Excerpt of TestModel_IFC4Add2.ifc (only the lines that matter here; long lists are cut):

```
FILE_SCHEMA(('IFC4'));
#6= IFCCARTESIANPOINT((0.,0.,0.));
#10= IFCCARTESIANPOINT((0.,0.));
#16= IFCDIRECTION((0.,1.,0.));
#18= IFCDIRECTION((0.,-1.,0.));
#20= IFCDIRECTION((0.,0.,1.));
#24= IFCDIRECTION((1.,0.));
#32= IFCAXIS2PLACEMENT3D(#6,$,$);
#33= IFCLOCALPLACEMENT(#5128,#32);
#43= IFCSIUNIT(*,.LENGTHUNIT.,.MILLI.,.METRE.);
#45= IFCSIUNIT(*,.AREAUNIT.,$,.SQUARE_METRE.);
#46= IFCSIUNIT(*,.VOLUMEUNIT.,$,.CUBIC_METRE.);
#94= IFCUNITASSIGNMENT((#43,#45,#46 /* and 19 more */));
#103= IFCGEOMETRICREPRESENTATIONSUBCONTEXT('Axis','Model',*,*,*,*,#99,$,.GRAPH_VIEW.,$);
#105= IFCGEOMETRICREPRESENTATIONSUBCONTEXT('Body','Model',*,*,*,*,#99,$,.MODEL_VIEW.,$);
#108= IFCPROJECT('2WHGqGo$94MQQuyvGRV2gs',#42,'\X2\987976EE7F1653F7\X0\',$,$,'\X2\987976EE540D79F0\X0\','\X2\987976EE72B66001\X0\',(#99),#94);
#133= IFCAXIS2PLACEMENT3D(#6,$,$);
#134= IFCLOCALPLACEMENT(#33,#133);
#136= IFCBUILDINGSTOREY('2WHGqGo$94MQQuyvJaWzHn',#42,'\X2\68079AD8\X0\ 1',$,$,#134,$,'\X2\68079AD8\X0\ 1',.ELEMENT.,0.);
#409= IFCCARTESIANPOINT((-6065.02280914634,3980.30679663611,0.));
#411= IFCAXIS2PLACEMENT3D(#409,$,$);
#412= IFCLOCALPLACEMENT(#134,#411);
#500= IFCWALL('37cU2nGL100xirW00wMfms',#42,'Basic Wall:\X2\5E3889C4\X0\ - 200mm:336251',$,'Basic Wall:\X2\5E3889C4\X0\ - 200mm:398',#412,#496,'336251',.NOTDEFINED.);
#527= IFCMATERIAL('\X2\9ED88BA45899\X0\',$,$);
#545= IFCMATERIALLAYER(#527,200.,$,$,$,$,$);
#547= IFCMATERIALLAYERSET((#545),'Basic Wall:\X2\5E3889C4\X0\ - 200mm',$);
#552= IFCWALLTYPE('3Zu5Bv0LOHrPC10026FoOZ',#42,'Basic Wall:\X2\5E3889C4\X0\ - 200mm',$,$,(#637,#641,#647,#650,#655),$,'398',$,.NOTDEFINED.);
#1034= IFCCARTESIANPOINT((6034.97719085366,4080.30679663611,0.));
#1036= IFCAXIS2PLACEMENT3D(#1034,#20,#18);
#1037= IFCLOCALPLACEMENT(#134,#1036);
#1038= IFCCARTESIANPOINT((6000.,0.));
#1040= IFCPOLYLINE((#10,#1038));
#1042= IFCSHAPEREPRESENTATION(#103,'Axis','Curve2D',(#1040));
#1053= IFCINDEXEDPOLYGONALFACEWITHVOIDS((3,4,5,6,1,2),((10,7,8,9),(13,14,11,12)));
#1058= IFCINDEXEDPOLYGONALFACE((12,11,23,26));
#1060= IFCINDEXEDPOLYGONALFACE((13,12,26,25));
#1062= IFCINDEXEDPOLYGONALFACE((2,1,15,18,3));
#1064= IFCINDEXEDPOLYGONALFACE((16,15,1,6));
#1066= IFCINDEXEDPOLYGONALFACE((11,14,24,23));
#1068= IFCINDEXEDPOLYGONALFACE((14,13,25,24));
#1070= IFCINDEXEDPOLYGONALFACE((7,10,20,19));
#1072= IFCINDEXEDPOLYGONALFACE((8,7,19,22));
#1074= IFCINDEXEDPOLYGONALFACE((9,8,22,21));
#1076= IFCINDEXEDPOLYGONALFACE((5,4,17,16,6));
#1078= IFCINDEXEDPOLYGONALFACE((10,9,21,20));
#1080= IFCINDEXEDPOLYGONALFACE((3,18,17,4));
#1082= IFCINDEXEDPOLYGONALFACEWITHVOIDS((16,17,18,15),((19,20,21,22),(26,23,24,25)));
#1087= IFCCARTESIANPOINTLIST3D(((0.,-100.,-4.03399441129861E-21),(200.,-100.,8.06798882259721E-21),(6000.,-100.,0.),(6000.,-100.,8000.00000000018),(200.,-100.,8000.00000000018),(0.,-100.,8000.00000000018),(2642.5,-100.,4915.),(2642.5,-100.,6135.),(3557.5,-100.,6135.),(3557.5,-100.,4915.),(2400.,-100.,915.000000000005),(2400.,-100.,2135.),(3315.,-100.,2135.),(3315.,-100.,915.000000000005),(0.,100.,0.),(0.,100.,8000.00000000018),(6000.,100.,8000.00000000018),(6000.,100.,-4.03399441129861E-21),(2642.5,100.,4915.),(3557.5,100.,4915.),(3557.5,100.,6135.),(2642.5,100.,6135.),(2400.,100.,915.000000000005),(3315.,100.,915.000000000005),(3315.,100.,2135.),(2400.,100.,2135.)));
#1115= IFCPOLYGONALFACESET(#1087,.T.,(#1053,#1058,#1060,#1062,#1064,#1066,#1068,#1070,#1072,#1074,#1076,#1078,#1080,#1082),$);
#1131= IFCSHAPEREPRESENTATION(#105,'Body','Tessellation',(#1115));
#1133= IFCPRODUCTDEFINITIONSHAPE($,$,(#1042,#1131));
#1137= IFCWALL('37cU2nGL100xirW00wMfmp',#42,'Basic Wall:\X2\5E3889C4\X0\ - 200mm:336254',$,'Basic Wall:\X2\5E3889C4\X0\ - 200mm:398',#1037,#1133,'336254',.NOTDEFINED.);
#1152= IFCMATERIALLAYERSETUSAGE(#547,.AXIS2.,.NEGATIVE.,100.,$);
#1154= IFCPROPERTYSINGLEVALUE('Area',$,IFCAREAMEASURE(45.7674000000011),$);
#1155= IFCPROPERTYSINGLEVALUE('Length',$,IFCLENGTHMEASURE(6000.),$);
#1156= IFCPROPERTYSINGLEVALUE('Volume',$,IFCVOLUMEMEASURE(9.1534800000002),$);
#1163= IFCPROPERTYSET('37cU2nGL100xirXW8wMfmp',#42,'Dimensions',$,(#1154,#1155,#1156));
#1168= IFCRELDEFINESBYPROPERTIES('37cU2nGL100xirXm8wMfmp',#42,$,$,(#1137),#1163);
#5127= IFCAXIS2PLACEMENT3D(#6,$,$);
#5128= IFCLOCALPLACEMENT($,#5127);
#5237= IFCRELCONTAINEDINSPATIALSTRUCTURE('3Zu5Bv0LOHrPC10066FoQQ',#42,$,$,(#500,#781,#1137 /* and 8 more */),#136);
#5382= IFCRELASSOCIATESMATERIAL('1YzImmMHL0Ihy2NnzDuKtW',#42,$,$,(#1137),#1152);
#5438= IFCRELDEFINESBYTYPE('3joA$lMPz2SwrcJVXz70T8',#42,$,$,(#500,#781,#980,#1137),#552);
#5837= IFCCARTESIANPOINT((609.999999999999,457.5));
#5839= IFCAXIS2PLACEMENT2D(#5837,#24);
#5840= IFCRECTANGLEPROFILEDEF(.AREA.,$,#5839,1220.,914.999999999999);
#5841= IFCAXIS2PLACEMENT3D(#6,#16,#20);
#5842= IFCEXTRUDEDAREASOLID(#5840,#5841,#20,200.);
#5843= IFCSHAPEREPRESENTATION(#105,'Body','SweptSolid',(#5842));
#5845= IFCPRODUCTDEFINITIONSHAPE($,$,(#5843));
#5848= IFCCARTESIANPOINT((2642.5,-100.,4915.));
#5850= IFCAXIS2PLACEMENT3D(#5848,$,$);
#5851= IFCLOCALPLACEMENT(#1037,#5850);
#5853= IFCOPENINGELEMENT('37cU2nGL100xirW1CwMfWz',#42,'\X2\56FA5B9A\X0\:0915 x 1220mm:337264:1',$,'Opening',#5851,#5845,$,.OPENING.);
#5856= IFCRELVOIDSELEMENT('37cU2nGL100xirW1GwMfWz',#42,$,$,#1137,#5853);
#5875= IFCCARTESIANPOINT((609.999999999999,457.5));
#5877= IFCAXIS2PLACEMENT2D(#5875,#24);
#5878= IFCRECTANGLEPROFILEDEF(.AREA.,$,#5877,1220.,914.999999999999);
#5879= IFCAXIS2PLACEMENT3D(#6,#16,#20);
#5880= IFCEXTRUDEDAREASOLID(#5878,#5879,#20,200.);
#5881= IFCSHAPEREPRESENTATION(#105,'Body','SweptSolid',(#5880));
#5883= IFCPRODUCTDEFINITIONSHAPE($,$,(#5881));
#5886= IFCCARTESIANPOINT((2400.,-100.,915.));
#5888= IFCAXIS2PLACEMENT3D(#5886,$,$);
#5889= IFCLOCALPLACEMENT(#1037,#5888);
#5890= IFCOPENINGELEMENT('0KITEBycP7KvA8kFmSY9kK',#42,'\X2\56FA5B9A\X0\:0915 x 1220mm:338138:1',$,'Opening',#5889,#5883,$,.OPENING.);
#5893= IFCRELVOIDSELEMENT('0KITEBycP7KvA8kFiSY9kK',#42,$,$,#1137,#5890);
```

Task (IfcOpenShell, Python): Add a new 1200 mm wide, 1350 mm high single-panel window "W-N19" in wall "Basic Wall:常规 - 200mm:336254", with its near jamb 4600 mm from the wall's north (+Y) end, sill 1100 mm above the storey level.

```python
import numpy as np
import ifcopenshell
import ifcopenshell.api.feature
import ifcopenshell.api.geometry
import ifcopenshell.api.pset
import ifcopenshell.api.root
import ifcopenshell.api.spatial
import ifcopenshell.geom
import ifcopenshell.util.element
import ifcopenshell.util.placement
import ifcopenshell.util.representation
import ifcopenshell.util.shape
import ifcopenshell.util.unit

model = ifcopenshell.open("TestModel_IFC4Add2.ifc")
unit_scale = ifcopenshell.util.unit.calculate_unit_scale(model)
area_scale = ifcopenshell.util.unit.calculate_unit_scale(model, "AREAUNIT")
volume_scale = ifcopenshell.util.unit.calculate_unit_scale(model, "VOLUMEUNIT")
settings = ifcopenshell.geom.settings()


def volume(element):
    """Net volume in cubic metres, openings subtracted."""
    shape = ifcopenshell.geom.create_shape(settings, element)
    return ifcopenshell.util.shape.get_volume(shape.geometry)


wall = model.by_guid("37cU2nGL100xirW00wMfmp")
storey = ifcopenshell.util.element.get_container(wall, ifc_class="IfcBuildingStorey")
context = ifcopenshell.util.representation.get_context(model, "Model", "Body", "MODEL_VIEW")
before = volume(wall)

width, height, from_end, sill = 1.2, 1.35, 4.6, 1.1  # metres

# The wall runs along its own X axis, and the end named is its -X end.
wall_shape = ifcopenshell.geom.create_shape(settings, wall)
x, y, z = ifcopenshell.util.shape.get_vertices(wall_shape.geometry).T
start = x.min() + from_end
face, thickness = float(y.min()), float(y.max() - y.min())
wall_matrix = ifcopenshell.util.placement.get_local_placement(wall.ObjectPlacement)
level = ifcopenshell.util.placement.get_local_placement(storey.ObjectPlacement)[2, 3]


def in_wall(x, y):
    """Placement at x, y metres in the wall's axes, at sill height."""
    matrix = wall_matrix.copy()
    matrix[:, 3] = wall_matrix @ np.array([x / unit_scale, y / unit_scale, 0.0, 1.0])
    matrix[2, 3] = level + sill / unit_scale
    return matrix


# Opening: a box that overshoots both wall faces by 50 mm.
opening = ifcopenshell.api.root.create_entity(model, ifc_class="IfcOpeningElement", predefined_type="OPENING")
box = ifcopenshell.api.geometry.add_wall_representation(
    model, context=context, length=width, height=height, thickness=thickness + 0.1
)
ifcopenshell.api.geometry.assign_representation(model, product=opening, representation=box)
ifcopenshell.api.geometry.edit_object_placement(model, product=opening, matrix=in_wall(start, face - 0.05), is_si=False)
ifcopenshell.api.feature.add_feature(model, feature=opening, element=wall)

window = ifcopenshell.api.root.create_entity(model, ifc_class="IfcWindow", name="W-N19", predefined_type="WINDOW")
window.OverallWidth, window.OverallHeight = width / unit_scale, height / unit_scale
window.PartitioningType = "SINGLE_PANEL"
body = ifcopenshell.api.geometry.add_window_representation(
    model,
    context=context,
    overall_width=window.OverallWidth,
    overall_height=window.OverallHeight,
    partition_type="SINGLE_PANEL",
)
ifcopenshell.api.geometry.assign_representation(model, product=window, representation=body)
ifcopenshell.api.spatial.assign_container(model, products=[window], relating_structure=storey)
ifcopenshell.api.feature.add_filling(model, opening=opening, element=window)

# Centre the window in the wall's thickness.
ifcopenshell.api.geometry.edit_object_placement(model, product=window, matrix=in_wall(start, face), is_si=False)
window_shape = ifcopenshell.geom.create_shape(settings, window)
depth = ifcopenshell.util.shape.get_vertices(window_shape.geometry)[:, 1]
offset = face + thickness / 2 - (depth.min() + depth.max()) / 2
ifcopenshell.api.geometry.edit_object_placement(model, product=window, matrix=in_wall(start, offset), is_si=False)

after = volume(wall)

# Update the wall's stored quantities.
pset = model.by_id(ifcopenshell.util.element.get_pset(wall, "Dimensions", should_inherit=False)["id"])
ifcopenshell.api.pset.edit_pset(model, pset=pset, properties={
    "Area": model.create_entity("IfcAreaMeasure", after / thickness / area_scale),
    "Volume": model.create_entity("IfcVolumeMeasure", after / volume_scale),
})

print(f"wall volume {before:.3f} -> {after:.3f} m3")

model.write("TestModel_IFC4Add2_updated.ifc")
```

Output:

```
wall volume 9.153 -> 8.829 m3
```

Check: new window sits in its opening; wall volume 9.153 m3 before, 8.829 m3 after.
